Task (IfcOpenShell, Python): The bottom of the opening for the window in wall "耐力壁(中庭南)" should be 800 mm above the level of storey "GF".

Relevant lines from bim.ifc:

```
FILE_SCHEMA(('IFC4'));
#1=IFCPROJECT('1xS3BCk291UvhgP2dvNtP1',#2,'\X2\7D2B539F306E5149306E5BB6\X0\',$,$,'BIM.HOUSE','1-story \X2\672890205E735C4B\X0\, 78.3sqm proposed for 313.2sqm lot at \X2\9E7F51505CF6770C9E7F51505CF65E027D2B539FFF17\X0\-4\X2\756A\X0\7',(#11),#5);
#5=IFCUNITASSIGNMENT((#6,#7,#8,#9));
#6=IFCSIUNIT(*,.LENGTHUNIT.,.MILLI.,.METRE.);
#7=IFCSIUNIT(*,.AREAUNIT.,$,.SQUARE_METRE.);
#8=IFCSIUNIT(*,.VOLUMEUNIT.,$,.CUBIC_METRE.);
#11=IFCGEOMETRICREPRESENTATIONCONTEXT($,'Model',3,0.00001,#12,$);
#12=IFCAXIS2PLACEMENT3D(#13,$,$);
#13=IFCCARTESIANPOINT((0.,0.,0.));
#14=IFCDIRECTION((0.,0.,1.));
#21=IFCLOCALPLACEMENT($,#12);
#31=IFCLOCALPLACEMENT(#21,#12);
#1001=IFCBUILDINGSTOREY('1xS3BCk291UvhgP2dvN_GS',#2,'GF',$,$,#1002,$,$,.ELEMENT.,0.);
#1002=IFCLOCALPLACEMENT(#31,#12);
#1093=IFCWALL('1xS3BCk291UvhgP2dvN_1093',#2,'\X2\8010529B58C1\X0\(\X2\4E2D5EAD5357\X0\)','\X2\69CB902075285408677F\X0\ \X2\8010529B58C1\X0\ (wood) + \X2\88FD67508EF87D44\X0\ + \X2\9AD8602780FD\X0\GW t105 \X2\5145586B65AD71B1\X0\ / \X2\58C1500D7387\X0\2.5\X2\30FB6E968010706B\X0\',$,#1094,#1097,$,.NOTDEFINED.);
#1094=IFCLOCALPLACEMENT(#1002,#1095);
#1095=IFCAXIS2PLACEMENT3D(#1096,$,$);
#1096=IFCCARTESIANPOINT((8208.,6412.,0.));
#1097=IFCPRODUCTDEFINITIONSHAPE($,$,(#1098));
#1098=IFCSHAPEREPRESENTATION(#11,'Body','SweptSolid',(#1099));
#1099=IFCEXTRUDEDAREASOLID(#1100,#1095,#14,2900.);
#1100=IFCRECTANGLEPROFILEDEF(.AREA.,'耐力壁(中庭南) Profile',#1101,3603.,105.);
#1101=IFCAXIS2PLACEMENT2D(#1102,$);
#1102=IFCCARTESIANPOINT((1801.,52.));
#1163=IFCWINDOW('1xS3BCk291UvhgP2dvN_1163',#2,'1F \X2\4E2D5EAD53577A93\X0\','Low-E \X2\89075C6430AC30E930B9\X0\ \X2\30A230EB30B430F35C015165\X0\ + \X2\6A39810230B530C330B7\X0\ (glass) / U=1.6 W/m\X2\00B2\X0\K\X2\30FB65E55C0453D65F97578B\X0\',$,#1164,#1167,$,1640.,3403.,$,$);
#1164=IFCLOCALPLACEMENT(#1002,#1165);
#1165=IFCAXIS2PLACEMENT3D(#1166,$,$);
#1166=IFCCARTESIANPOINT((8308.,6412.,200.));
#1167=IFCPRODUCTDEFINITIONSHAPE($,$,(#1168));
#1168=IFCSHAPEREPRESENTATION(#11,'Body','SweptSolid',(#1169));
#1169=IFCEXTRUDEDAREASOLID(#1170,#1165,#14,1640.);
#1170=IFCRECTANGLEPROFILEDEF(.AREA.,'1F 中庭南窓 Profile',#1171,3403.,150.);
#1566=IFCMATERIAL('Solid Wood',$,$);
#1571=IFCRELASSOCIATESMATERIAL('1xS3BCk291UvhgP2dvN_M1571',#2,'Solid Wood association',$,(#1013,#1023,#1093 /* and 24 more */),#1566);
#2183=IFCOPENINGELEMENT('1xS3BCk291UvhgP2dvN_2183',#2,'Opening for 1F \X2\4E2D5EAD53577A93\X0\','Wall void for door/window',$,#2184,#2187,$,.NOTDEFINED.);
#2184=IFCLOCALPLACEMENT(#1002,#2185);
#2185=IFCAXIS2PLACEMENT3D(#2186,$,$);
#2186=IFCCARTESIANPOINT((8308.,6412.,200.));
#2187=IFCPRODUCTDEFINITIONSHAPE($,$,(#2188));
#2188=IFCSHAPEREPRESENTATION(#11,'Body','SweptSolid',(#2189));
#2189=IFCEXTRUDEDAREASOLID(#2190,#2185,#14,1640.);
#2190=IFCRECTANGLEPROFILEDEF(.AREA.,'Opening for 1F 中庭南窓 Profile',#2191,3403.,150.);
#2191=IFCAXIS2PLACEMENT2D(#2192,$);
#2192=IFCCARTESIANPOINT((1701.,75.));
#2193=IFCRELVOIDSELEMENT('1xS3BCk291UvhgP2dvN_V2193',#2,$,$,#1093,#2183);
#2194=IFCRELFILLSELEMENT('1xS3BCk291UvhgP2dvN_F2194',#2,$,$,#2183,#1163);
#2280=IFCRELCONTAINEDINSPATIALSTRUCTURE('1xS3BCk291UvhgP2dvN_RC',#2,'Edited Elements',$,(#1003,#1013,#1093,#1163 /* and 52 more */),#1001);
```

```python
import numpy as np
import ifcopenshell
import ifcopenshell.api.geometry
import ifcopenshell.geom
import ifcopenshell.util.element
import ifcopenshell.util.placement
import ifcopenshell.util.shape
import ifcopenshell.util.unit

model = ifcopenshell.open("bim.ifc")
unit_scale = ifcopenshell.util.unit.calculate_unit_scale(model)

window = model.by_guid("1xS3BCk291UvhgP2dvN_1163")
opening = window.FillsVoids[0].RelatingOpeningElement
storey = ifcopenshell.util.element.get_container(window, ifc_class="IfcBuildingStorey")
level = ifcopenshell.util.placement.get_local_placement(storey.ObjectPlacement)[2, 3]

# The opening's origin need not be at the sill, so measure its lowest point.
shape = ifcopenshell.geom.create_shape(ifcopenshell.geom.settings(), opening)
bottom = ifcopenshell.util.shape.get_shape_bottom_elevation(shape, shape.geometry) / unit_scale
dz = level + 0.8 / unit_scale - bottom

shift = np.array([0.0, 0.0, dz])
# The window is not placed relative to its opening, so move both.
for product in (opening, window):
    matrix = ifcopenshell.util.placement.get_local_placement(product.ObjectPlacement)
    matrix[:3, 3] += shift
    ifcopenshell.api.geometry.edit_object_placement(model, product=product, matrix=matrix, is_si=False)

print(f"moved by {dz * unit_scale:+.3f} m")

model.write("bim_edited.ifc")
```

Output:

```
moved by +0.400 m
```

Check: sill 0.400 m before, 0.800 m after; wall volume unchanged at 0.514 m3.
